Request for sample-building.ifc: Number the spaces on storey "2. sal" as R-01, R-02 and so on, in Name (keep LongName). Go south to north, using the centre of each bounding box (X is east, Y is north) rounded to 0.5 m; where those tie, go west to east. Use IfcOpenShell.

First a look at what the model holds.

```python
import ifcopenshell
import ifcopenshell.util.element
import ifcopenshell.util.placement

model = ifcopenshell.open("sample-building.ifc")
print(model.schema)
storey = next(s for s in model.by_type("IfcBuildingStorey") if s.Name == "2. sal")
spaces = [e for e in ifcopenshell.util.element.get_decomposition(storey) if e.is_a("IfcSpace")]
for e in sorted(spaces, key=lambda e: e.id()):
    origin = ifcopenshell.util.placement.get_local_placement(e.ObjectPlacement)[:3, 3]
    print(e.id(), e.Name, e.LongName, origin.round(2) + 0.0, sep=" | ")
```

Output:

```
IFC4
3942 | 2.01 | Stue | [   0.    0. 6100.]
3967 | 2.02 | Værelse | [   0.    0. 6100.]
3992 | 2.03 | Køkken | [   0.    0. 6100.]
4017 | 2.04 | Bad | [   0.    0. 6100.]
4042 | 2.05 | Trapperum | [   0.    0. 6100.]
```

```python
import ifcopenshell
import ifcopenshell.geom
import ifcopenshell.util.element
import ifcopenshell.util.shape

model = ifcopenshell.open("sample-building.ifc")
settings = ifcopenshell.geom.settings()
settings.set("use-world-coords", True)


def centre(element):
    shape = ifcopenshell.geom.create_shape(settings, element)
    return ifcopenshell.util.shape.get_bbox_centroid(shape.geometry)


storey = next(s for s in model.by_type("IfcBuildingStorey") if s.Name == "2. sal")
spaces = [e for e in ifcopenshell.util.element.get_decomposition(storey) if e.is_a("IfcSpace")]

# Insertion points can sit at a corner or the storey origin, so sort by the geometry (in metres).
centres = {e: centre(e) for e in spaces}
spaces.sort(key=lambda e: (round(centres[e][1] / 0.5), centres[e][0]))

for i, e in enumerate(spaces, start=1):
    number = f"R-{i:02d}"
    e.Name = number
    print(e.id(), number)

model.write("sample-building_v2.ifc")
```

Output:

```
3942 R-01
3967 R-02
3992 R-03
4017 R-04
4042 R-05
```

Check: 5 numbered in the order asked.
